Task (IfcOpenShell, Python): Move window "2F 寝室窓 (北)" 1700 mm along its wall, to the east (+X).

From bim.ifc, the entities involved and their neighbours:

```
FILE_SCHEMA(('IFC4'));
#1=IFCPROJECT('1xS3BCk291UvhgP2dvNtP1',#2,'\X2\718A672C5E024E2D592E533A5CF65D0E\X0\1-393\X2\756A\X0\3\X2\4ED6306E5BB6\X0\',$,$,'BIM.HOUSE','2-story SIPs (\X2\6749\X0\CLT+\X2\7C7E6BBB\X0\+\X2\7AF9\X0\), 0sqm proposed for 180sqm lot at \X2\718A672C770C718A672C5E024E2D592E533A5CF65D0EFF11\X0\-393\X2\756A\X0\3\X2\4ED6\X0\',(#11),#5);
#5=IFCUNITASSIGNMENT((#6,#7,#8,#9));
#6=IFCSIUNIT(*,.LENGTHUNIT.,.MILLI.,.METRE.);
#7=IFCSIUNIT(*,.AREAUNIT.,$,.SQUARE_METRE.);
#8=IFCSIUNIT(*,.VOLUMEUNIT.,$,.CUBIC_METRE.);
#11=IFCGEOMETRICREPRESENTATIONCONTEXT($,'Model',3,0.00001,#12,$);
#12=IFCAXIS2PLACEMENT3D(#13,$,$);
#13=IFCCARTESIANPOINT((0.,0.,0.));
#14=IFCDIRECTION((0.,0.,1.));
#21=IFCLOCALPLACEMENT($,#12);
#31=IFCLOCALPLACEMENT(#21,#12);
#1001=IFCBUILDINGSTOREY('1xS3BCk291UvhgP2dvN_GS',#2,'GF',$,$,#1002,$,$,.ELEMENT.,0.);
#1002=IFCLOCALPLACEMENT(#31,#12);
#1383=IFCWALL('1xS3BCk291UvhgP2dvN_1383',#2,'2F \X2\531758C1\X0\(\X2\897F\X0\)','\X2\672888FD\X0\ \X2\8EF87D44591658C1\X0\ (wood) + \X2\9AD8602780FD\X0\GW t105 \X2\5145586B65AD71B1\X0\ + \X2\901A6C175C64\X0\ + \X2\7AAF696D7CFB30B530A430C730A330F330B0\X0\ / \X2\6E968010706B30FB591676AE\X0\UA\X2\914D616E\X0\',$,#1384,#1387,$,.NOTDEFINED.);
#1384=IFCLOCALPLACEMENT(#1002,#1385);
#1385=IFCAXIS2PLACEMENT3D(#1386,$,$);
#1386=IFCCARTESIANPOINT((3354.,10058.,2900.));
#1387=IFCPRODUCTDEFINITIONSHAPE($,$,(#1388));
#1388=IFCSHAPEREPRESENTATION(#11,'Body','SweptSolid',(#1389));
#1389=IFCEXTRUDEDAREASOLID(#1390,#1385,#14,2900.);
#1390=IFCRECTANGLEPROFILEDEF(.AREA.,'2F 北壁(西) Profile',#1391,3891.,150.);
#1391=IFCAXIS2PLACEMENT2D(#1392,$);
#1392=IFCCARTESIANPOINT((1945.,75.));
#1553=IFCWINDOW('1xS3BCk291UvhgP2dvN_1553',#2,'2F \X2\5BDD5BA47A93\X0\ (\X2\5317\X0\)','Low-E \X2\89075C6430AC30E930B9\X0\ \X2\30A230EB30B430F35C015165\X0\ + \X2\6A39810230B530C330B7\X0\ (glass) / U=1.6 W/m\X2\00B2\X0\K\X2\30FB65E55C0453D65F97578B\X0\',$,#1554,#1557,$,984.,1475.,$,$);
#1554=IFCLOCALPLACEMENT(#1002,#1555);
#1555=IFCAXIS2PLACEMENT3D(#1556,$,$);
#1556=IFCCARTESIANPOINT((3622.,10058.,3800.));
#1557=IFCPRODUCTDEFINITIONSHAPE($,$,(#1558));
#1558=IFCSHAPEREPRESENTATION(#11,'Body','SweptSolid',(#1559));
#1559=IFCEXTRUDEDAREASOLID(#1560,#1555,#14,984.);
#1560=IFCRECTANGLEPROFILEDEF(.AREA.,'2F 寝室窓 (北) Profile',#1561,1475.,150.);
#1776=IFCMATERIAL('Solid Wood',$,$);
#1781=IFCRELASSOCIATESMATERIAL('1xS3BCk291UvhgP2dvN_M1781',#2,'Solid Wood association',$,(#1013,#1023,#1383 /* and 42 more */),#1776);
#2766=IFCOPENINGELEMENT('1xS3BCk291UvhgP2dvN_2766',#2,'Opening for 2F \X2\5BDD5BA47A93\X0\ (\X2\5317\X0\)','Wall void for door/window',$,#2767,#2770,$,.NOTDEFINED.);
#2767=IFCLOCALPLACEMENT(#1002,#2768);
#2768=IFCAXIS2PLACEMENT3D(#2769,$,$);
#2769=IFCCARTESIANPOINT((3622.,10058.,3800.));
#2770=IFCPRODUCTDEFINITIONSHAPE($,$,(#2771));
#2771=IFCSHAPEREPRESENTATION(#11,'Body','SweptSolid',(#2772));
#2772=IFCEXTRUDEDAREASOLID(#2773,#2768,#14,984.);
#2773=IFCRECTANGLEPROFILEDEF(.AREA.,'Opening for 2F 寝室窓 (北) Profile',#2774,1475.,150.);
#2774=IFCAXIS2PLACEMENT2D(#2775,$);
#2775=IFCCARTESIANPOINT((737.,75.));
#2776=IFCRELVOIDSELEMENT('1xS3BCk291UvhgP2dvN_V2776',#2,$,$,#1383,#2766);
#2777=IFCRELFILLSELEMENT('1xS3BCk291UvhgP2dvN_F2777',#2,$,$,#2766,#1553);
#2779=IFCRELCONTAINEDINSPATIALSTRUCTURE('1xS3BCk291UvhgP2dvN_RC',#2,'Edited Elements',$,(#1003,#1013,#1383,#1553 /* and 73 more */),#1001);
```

```python
import ifcopenshell
import ifcopenshell.api.geometry
import ifcopenshell.util.placement
import ifcopenshell.util.unit

model = ifcopenshell.open("bim.ifc")
unit_scale = ifcopenshell.util.unit.calculate_unit_scale(model)

window = model.by_guid("1xS3BCk291UvhgP2dvN_1553")
opening = window.FillsVoids[0].RelatingOpeningElement
wall = opening.VoidsElements[0].RelatingBuildingElement

wall_matrix = ifcopenshell.util.placement.get_local_placement(wall.ObjectPlacement)
shift = wall_matrix[:3, 0] * 1.7 / unit_scale
before = ifcopenshell.util.placement.get_local_placement(window.ObjectPlacement)[:3, 3].copy()

# The window is not placed relative to its opening, so move both.
for product in (opening, window):
    matrix = ifcopenshell.util.placement.get_local_placement(product.ObjectPlacement)
    matrix[:3, 3] += shift
    ifcopenshell.api.geometry.edit_object_placement(model, product=product, matrix=matrix, is_si=False)

after = ifcopenshell.util.placement.get_local_placement(window.ObjectPlacement)[:3, 3]
print("window moved by", (after - before).round(3) + 0.0)

model.write("bim_updated.ifc")
```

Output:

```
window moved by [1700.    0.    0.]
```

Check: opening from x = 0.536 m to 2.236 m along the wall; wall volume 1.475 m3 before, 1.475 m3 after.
